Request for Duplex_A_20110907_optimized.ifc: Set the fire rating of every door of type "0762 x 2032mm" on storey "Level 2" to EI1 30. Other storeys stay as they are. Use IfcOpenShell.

First a look at what the model holds.

```python
import ifcopenshell
import ifcopenshell.util.element

model = ifcopenshell.open("Duplex_A_20110907_optimized.ifc")
print(model.schema)
storey = next(s for s in model.by_type("IfcBuildingStorey") if s.Name == "Level 2")
doors = [e for e in ifcopenshell.util.element.get_decomposition(storey) if e.is_a("IfcDoor")]
seen = {}
for e in doors:
    element_type = ifcopenshell.util.element.get_type(e)
    key = (element_type.Name if element_type != e and element_type else None, ifcopenshell.util.element.get_pset(e, "Pset_DoorCommon", "FireRating"))
    seen[key] = seen.get(key, 0) + 1
for (name, value), count in sorted(seen.items(), key=str):
    print(count, "x", name, "|", value)
```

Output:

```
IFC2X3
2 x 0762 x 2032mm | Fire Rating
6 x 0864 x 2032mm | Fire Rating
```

```python
import ifcopenshell
import ifcopenshell.api.pset
import ifcopenshell.util.element

model = ifcopenshell.open("Duplex_A_20110907_optimized.ifc")

storey = next(s for s in model.by_type("IfcBuildingStorey") if s.Name == "Level 2")
doors = [e for e in ifcopenshell.util.element.get_decomposition(storey) if e.is_a("IfcDoor")]

count = 0
for e in doors:
    element_type = ifcopenshell.util.element.get_type(e)
    if element_type in (None, e) or element_type.Name != "0762 x 2032mm":
        continue
    # add_pset returns the element's existing set when there is one.
    pset = ifcopenshell.api.pset.add_pset(model, product=e, name="Pset_DoorCommon")
    ifcopenshell.api.pset.edit_pset(model, pset=pset, properties={"FireRating": "EI1 30"})
    count += 1

print(count, "doors updated")

model.write("Duplex_A_20110907_optimized_rev.ifc")
```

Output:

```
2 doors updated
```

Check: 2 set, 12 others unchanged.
